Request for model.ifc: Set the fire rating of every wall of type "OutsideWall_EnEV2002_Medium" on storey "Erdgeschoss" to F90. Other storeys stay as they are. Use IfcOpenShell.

First a look at what the model holds.

```python
import ifcopenshell
import ifcopenshell.util.element

model = ifcopenshell.open("model.ifc")
print(model.schema)
storey = next(s for s in model.by_type("IfcBuildingStorey") if s.Name == "Erdgeschoss")
walls = [e for e in ifcopenshell.util.element.get_decomposition(storey) if e.is_a("IfcWall")]
seen = {}
for e in walls:
    element_type = ifcopenshell.util.element.get_type(e)
    key = (element_type.Name if element_type != e and element_type else None, ifcopenshell.util.element.get_pset(e, "Pset_WallCommon", "FireRating"))
    seen[key] = seen.get(key, 0) + 1
for (name, value), count in sorted(seen.items(), key=str):
    print(count, "x", name, "|", value)
```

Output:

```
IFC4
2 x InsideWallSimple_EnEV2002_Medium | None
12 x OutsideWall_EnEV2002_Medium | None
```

```python
import ifcopenshell
import ifcopenshell.api.pset
import ifcopenshell.util.element

model = ifcopenshell.open("model.ifc")

storey = next(s for s in model.by_type("IfcBuildingStorey") if s.Name == "Erdgeschoss")
walls = [e for e in ifcopenshell.util.element.get_decomposition(storey) if e.is_a("IfcWall")]

count = 0
for e in walls:
    element_type = ifcopenshell.util.element.get_type(e)
    if element_type in (None, e) or element_type.Name != "OutsideWall_EnEV2002_Medium":
        continue
    # add_pset returns the element's existing set when there is one.
    pset = ifcopenshell.api.pset.add_pset(model, product=e, name="Pset_WallCommon")
    ifcopenshell.api.pset.edit_pset(model, pset=pset, properties={"FireRating": "F90"})
    count += 1

print(count, "walls updated")

model.write("model_edited.ifc")
```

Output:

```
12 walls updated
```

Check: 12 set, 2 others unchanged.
